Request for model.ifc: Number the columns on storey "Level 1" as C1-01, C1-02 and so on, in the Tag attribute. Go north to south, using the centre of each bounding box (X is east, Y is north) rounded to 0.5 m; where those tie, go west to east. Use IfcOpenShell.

First a look at what the model holds.

```python
import ifcopenshell
import ifcopenshell.util.element
import ifcopenshell.util.placement

model = ifcopenshell.open("model.ifc")
print(model.schema)
storey = next(s for s in model.by_type("IfcBuildingStorey") if s.Name == "Level 1")
columns = [e for e in ifcopenshell.util.element.get_decomposition(storey) if e.is_a("IfcColumn")]
for e in sorted(columns, key=lambda e: e.id()):
    origin = ifcopenshell.util.placement.get_local_placement(e.ObjectPlacement)[:3, 3]
    print(e.id(), e.Tag, e.Name, origin.round(2) + 0.0, sep=" | ")
```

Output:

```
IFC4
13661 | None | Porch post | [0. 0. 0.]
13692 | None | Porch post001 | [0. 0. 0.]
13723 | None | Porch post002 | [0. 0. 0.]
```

```python
import ifcopenshell
import ifcopenshell.geom
import ifcopenshell.util.element
import ifcopenshell.util.shape

model = ifcopenshell.open("model.ifc")
settings = ifcopenshell.geom.settings()
settings.set("use-world-coords", True)


def centre(element):
    shape = ifcopenshell.geom.create_shape(settings, element)
    return ifcopenshell.util.shape.get_bbox_centroid(shape.geometry)


storey = next(s for s in model.by_type("IfcBuildingStorey") if s.Name == "Level 1")
columns = [e for e in ifcopenshell.util.element.get_decomposition(storey) if e.is_a("IfcColumn")]

# Insertion points can sit at a corner or the storey origin, so sort by the geometry (in metres).
centres = {e: centre(e) for e in columns}
columns.sort(key=lambda e: (-round(centres[e][1] / 0.5), centres[e][0]))

for i, e in enumerate(columns, start=1):
    number = f"C1-{i:02d}"
    e.Tag = number
    print(e.id(), number)

model.write("model_v2.ifc")
```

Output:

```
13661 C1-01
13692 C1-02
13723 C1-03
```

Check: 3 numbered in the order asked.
